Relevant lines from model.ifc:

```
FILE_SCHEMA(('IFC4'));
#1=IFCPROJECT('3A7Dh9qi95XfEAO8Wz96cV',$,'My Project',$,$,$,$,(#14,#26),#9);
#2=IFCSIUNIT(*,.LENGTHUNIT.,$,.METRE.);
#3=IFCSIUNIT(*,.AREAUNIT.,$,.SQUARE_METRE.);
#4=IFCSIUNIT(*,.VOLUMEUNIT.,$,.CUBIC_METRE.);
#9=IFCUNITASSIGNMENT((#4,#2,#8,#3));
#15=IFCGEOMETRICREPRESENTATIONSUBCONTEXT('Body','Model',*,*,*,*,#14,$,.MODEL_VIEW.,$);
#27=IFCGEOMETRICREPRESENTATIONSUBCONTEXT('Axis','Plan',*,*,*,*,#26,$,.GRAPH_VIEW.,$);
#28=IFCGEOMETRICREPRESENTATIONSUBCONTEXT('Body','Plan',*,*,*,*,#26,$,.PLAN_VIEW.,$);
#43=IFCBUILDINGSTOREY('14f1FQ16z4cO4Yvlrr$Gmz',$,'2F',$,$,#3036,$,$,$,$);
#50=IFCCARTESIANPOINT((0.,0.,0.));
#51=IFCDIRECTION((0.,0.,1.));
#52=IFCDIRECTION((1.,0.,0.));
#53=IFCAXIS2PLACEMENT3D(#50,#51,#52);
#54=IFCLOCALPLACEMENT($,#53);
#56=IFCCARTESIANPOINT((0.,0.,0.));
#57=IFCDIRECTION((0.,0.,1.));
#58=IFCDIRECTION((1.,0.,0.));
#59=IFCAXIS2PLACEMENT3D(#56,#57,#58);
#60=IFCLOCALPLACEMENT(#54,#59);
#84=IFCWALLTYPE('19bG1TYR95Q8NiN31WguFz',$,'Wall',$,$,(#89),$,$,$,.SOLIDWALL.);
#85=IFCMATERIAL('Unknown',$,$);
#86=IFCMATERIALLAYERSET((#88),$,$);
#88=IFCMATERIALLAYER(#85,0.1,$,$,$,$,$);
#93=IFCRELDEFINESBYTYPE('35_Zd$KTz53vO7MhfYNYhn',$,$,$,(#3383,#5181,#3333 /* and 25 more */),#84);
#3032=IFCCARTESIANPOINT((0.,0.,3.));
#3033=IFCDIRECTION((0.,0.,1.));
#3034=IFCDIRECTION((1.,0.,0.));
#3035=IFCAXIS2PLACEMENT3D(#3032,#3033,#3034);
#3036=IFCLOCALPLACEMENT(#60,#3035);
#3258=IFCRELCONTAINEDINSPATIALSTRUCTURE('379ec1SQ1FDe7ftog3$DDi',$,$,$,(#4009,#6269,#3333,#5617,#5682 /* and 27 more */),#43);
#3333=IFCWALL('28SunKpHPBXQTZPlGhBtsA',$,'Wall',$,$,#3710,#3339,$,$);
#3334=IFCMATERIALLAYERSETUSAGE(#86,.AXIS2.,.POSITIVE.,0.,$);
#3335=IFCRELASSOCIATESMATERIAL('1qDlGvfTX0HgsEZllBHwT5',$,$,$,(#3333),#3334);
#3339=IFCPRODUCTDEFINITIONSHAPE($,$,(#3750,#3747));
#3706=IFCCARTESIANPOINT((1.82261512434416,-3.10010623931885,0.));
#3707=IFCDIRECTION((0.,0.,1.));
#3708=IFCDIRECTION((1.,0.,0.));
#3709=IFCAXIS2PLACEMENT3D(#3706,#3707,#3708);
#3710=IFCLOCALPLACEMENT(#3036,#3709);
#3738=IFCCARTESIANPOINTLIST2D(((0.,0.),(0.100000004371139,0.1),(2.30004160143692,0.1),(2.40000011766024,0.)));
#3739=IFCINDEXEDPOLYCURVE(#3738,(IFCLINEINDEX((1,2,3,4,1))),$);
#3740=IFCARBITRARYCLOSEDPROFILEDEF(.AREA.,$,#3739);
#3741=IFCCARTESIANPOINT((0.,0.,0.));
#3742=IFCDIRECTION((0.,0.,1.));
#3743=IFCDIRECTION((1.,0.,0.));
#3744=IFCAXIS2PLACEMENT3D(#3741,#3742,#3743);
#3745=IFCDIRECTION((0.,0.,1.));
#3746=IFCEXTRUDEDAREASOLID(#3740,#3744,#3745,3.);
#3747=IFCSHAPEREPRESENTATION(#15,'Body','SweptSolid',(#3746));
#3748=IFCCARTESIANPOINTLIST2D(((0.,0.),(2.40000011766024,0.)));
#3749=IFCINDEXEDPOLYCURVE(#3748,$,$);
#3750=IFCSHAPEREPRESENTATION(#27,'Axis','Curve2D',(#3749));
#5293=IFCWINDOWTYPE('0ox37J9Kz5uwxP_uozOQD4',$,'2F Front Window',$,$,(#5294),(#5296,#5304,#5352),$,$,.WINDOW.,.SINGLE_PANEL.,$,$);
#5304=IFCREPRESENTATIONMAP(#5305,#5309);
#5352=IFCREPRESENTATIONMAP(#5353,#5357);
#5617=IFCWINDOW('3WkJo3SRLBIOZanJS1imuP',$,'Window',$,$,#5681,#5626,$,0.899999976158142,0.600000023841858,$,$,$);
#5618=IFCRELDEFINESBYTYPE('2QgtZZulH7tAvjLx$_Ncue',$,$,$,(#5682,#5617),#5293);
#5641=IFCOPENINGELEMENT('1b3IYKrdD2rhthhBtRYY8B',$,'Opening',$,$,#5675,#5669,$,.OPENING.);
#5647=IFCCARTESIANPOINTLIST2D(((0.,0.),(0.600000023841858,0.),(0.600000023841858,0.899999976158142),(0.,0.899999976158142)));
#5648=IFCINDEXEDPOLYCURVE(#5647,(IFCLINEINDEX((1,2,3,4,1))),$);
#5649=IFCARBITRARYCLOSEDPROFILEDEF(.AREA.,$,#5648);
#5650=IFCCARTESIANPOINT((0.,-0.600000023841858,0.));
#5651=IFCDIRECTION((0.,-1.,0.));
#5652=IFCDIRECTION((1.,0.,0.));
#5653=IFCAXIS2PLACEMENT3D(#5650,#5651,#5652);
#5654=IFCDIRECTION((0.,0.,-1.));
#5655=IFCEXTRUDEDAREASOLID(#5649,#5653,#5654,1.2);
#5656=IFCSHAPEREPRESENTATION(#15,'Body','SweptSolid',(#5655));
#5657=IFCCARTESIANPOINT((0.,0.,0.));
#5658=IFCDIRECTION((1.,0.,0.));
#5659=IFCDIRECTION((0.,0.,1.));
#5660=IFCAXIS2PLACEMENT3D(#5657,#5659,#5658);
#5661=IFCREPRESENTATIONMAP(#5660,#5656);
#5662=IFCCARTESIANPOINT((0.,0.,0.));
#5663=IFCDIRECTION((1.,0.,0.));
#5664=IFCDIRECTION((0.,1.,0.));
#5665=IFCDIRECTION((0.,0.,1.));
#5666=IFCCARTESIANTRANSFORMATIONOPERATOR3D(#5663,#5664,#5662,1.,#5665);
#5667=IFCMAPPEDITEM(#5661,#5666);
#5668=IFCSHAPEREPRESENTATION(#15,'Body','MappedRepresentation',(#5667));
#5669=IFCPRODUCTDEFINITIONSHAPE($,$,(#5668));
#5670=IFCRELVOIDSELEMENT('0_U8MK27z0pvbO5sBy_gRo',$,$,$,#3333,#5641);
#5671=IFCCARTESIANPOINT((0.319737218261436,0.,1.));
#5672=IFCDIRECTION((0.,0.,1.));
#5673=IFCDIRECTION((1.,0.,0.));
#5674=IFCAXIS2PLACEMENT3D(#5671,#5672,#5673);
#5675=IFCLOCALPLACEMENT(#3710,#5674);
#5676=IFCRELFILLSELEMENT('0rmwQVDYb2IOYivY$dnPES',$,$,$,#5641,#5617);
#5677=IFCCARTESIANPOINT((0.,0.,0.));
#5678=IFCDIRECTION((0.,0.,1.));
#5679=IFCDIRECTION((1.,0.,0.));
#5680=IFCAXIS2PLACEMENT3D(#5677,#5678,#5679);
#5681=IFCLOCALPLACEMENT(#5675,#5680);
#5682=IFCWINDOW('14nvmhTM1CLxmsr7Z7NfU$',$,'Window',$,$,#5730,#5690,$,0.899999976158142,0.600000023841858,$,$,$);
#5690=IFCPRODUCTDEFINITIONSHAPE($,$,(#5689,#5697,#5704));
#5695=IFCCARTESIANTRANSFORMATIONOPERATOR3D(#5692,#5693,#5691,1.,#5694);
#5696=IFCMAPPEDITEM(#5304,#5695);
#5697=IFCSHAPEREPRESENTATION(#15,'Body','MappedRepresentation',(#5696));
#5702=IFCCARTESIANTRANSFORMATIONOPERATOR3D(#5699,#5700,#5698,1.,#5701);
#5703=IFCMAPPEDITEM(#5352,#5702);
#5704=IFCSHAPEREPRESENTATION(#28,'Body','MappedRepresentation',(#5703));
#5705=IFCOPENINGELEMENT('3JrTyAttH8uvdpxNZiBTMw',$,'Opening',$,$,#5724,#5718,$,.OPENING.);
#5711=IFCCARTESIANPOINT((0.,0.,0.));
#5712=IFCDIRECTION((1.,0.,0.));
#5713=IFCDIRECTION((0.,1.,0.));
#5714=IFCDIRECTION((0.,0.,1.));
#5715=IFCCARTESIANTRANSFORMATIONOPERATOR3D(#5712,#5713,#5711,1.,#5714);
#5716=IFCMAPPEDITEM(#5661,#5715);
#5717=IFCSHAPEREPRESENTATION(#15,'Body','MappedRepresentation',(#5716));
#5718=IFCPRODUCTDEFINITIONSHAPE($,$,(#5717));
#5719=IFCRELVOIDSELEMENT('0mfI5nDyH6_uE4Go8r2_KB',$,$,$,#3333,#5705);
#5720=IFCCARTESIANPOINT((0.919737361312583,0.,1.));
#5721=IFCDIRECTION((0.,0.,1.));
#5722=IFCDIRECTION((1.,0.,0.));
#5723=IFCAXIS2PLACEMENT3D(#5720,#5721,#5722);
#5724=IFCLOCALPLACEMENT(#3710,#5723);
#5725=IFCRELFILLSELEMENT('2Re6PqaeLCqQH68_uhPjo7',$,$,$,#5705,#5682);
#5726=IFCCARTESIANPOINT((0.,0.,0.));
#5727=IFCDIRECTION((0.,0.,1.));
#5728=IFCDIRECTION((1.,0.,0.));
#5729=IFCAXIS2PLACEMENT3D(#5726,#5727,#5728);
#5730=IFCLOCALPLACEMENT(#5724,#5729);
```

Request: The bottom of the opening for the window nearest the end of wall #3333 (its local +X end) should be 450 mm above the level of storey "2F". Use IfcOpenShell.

```python
import numpy as np
import ifcopenshell
import ifcopenshell.api.geometry
import ifcopenshell.geom
import ifcopenshell.util.element
import ifcopenshell.util.placement
import ifcopenshell.util.shape
import ifcopenshell.util.unit

model = ifcopenshell.open("model.ifc")
unit_scale = ifcopenshell.util.unit.calculate_unit_scale(model)

window = model.by_guid("14nvmhTM1CLxmsr7Z7NfU$")
opening = window.FillsVoids[0].RelatingOpeningElement
storey = ifcopenshell.util.element.get_container(window, ifc_class="IfcBuildingStorey")
level = ifcopenshell.util.placement.get_local_placement(storey.ObjectPlacement)[2, 3]

# The opening's origin need not be at the sill, so measure its lowest point.
shape = ifcopenshell.geom.create_shape(ifcopenshell.geom.settings(), opening)
bottom = ifcopenshell.util.shape.get_shape_bottom_elevation(shape, shape.geometry) / unit_scale
dz = level + 0.45 / unit_scale - bottom

shift = np.array([0.0, 0.0, dz])
# The window is placed relative to its opening, so it follows when the opening moves.
matrix = ifcopenshell.util.placement.get_local_placement(opening.ObjectPlacement)
matrix[:3, 3] += shift
ifcopenshell.api.geometry.edit_object_placement(
    model, product=opening, matrix=matrix, is_si=False, should_transform_children=True
)

print(f"moved by {dz * unit_scale:+.3f} m")

model.write("model-out.ifc")
```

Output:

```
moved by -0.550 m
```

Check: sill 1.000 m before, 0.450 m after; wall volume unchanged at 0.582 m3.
